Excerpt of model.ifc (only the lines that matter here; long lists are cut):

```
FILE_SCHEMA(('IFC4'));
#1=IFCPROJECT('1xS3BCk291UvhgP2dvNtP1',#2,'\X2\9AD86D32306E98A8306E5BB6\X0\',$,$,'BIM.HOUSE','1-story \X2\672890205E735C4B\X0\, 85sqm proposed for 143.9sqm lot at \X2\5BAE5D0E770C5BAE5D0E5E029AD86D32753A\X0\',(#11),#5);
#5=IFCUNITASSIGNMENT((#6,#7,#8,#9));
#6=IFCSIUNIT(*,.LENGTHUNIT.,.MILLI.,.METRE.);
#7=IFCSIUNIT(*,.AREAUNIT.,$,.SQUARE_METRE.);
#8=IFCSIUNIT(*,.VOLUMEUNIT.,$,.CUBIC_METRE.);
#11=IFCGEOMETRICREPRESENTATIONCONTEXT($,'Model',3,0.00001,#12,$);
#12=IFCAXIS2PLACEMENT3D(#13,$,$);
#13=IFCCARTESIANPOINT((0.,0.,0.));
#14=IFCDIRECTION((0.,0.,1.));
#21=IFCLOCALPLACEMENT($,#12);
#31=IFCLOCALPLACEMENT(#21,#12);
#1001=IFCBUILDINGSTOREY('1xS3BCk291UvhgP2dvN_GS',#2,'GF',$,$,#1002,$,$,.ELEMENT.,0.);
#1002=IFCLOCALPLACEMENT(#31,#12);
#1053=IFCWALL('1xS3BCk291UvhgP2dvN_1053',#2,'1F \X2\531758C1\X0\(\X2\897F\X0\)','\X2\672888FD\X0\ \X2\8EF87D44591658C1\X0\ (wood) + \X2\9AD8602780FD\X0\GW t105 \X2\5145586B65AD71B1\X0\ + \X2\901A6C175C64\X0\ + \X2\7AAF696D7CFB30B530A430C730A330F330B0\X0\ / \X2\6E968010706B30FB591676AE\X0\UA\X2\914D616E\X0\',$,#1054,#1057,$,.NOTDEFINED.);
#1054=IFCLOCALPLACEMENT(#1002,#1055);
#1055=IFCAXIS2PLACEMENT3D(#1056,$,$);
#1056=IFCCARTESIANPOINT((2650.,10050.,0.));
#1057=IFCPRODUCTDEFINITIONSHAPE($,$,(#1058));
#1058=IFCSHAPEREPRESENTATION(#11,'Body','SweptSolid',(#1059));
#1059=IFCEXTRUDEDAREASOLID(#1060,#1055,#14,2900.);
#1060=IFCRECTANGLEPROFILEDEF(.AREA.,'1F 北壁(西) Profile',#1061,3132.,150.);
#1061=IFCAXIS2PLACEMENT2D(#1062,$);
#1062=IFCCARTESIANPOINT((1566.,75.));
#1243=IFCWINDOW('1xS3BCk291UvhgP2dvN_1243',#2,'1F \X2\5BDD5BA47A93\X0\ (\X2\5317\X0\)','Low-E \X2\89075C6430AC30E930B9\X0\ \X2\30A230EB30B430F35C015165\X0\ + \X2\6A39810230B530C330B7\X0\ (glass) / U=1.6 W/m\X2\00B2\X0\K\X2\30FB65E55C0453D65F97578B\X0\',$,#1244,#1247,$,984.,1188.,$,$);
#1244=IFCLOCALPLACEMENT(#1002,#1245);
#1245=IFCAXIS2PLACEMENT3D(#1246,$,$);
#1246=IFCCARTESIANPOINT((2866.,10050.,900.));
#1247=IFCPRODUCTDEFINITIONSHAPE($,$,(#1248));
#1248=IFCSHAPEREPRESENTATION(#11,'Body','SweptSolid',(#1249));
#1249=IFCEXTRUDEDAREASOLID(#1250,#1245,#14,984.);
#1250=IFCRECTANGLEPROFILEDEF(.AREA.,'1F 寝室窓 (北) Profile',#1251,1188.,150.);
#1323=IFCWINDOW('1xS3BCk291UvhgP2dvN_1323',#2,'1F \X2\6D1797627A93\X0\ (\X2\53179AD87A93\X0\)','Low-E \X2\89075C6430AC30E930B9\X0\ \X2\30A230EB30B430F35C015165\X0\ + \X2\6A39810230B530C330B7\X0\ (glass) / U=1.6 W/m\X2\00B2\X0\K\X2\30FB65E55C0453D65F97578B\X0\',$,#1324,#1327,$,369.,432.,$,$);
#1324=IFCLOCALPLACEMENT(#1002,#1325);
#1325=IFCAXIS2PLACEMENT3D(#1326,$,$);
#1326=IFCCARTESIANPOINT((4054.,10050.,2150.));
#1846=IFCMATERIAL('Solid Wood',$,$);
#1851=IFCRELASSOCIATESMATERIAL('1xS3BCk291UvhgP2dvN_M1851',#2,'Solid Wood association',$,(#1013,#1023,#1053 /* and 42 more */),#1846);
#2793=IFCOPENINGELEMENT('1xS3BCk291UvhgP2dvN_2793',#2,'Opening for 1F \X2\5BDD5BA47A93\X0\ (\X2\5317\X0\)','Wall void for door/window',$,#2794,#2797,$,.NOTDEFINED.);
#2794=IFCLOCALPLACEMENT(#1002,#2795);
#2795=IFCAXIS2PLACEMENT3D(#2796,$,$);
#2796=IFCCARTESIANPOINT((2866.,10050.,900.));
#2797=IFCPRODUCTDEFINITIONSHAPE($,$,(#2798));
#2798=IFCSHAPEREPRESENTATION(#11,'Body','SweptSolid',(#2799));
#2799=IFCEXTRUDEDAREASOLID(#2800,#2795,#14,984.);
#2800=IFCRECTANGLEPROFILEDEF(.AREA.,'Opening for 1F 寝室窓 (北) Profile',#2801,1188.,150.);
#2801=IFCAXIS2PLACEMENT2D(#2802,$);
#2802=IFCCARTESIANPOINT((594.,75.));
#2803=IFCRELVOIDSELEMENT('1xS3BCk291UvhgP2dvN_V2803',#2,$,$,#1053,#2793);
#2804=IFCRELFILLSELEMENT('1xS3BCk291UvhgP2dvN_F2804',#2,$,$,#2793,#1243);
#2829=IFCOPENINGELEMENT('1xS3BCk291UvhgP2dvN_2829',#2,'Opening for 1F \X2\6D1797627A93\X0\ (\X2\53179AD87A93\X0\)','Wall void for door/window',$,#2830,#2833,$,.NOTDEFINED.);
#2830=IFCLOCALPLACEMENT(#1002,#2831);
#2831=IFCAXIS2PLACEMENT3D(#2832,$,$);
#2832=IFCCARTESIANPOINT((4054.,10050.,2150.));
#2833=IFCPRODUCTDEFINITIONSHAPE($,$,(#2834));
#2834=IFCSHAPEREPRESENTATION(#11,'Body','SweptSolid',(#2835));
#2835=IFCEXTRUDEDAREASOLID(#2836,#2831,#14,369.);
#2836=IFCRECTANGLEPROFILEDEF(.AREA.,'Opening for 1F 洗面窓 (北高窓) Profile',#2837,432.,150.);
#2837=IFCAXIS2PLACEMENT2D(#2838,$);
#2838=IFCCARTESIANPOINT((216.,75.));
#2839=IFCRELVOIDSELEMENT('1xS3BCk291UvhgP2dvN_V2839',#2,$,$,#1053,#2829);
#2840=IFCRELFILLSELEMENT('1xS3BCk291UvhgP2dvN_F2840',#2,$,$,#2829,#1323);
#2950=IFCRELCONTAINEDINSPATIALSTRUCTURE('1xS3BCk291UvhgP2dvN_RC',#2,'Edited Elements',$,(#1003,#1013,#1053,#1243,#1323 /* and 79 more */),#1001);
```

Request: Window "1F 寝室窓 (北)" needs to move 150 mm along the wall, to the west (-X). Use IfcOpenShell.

```python
import ifcopenshell
import ifcopenshell.api.geometry
import ifcopenshell.util.placement
import ifcopenshell.util.unit

model = ifcopenshell.open("model.ifc")
unit_scale = ifcopenshell.util.unit.calculate_unit_scale(model)

window = model.by_guid("1xS3BCk291UvhgP2dvN_1243")
opening = window.FillsVoids[0].RelatingOpeningElement
wall = opening.VoidsElements[0].RelatingBuildingElement

wall_matrix = ifcopenshell.util.placement.get_local_placement(wall.ObjectPlacement)
shift = wall_matrix[:3, 0] * -0.15 / unit_scale
before = ifcopenshell.util.placement.get_local_placement(window.ObjectPlacement)[:3, 3].copy()

# The window is not placed relative to its opening, so move both.
for product in (opening, window):
    matrix = ifcopenshell.util.placement.get_local_placement(product.ObjectPlacement)
    matrix[:3, 3] += shift
    ifcopenshell.api.geometry.edit_object_placement(model, product=product, matrix=matrix, is_si=False)

after = ifcopenshell.util.placement.get_local_placement(window.ObjectPlacement)[:3, 3]
print("window moved by", (after - before).round(3) + 0.0)

model.write("model-out.ifc")
```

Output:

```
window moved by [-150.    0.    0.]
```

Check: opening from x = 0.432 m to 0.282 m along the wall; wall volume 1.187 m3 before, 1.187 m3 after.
